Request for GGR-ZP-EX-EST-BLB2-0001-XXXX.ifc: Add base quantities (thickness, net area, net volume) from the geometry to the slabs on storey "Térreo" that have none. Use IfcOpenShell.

First a look at what the model holds.

```python
import ifcopenshell
import ifcopenshell.util.element
import ifcopenshell.util.unit

model = ifcopenshell.open("GGR-ZP-EX-EST-BLB2-0001-XXXX.ifc")
print(model.schema)
for unit_type in ("LENGTHUNIT", "AREAUNIT", "VOLUMEUNIT"):
    print(unit_type, ifcopenshell.util.unit.calculate_unit_scale(model, unit_type))
storey = next(s for s in model.by_type("IfcBuildingStorey") if s.Name == "Térreo")
slabs = [e for e in ifcopenshell.util.element.get_decomposition(storey) if e.is_a("IfcSlab")]
for e in sorted(slabs, key=lambda e: e.id()):
    print(e.id(), e.is_a(), e.Name, list(ifcopenshell.util.element.get_psets(e, qtos_only=True)), sep=" | ")
```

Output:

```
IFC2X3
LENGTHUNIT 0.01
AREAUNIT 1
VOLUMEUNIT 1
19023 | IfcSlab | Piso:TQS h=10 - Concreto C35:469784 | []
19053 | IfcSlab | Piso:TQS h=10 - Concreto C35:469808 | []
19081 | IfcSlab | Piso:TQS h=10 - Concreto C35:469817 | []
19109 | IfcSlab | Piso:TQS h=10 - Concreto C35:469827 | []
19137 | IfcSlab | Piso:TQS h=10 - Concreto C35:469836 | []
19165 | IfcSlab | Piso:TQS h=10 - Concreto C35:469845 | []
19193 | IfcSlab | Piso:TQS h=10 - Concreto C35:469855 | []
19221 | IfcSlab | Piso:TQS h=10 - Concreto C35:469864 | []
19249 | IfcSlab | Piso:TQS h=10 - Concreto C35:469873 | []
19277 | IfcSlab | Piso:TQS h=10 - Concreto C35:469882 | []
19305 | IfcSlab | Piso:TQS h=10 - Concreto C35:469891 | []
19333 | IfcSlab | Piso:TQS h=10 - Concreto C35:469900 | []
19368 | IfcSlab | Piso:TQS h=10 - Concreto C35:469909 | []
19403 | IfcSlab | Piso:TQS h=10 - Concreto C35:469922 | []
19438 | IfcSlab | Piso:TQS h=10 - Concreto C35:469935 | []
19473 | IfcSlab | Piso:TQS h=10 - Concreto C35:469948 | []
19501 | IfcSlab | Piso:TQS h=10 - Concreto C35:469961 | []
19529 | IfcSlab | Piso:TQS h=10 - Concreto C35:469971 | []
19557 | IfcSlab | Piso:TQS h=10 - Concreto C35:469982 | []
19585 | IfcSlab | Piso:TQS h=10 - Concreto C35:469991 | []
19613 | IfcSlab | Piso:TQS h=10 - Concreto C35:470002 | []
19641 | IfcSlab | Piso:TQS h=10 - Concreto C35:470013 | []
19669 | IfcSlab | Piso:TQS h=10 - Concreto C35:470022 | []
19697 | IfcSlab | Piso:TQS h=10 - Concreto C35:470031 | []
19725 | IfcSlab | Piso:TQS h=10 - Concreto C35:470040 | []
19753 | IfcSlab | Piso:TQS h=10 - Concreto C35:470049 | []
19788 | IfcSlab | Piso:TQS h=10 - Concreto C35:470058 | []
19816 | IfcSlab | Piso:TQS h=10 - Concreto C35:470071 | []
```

```python
import ifcopenshell
import ifcopenshell.api.pset
import ifcopenshell.geom
import ifcopenshell.util.element
import ifcopenshell.util.shape
import ifcopenshell.util.unit

model = ifcopenshell.open("GGR-ZP-EX-EST-BLB2-0001-XXXX.ifc")
unit_scale = ifcopenshell.util.unit.calculate_unit_scale(model)
area_scale = ifcopenshell.util.unit.calculate_unit_scale(model, "AREAUNIT")
volume_scale = ifcopenshell.util.unit.calculate_unit_scale(model, "VOLUMEUNIT")
settings = ifcopenshell.geom.settings()

storey = next(s for s in model.by_type("IfcBuildingStorey") if s.Name == "Térreo")
slabs = [e for e in ifcopenshell.util.element.get_decomposition(storey) if e.is_a("IfcSlab")]

for e in sorted(slabs, key=lambda e: e.id()):
    if ifcopenshell.util.element.get_psets(e, qtos_only=True, should_inherit=False):
        continue
    # Geometry comes back in metres, in the element's own axes.
    shape = ifcopenshell.geom.create_shape(settings, e)
    values = {
        "Width": ifcopenshell.util.shape.get_z(shape.geometry) / unit_scale,
        "NetArea": ifcopenshell.util.shape.get_footprint_area(shape.geometry) / area_scale,
        "NetVolume": ifcopenshell.util.shape.get_volume(shape.geometry) / volume_scale,
    }
    qto = ifcopenshell.api.pset.add_qto(model, product=e, name="BaseQuantities")
    ifcopenshell.api.pset.edit_qto(model, qto=qto, properties=values)
    print(e.id(), {k: round(v, 3) for k, v in values.items()})

model.write("GGR-ZP-EX-EST-BLB2-0001-XXXX_edited.ifc")
```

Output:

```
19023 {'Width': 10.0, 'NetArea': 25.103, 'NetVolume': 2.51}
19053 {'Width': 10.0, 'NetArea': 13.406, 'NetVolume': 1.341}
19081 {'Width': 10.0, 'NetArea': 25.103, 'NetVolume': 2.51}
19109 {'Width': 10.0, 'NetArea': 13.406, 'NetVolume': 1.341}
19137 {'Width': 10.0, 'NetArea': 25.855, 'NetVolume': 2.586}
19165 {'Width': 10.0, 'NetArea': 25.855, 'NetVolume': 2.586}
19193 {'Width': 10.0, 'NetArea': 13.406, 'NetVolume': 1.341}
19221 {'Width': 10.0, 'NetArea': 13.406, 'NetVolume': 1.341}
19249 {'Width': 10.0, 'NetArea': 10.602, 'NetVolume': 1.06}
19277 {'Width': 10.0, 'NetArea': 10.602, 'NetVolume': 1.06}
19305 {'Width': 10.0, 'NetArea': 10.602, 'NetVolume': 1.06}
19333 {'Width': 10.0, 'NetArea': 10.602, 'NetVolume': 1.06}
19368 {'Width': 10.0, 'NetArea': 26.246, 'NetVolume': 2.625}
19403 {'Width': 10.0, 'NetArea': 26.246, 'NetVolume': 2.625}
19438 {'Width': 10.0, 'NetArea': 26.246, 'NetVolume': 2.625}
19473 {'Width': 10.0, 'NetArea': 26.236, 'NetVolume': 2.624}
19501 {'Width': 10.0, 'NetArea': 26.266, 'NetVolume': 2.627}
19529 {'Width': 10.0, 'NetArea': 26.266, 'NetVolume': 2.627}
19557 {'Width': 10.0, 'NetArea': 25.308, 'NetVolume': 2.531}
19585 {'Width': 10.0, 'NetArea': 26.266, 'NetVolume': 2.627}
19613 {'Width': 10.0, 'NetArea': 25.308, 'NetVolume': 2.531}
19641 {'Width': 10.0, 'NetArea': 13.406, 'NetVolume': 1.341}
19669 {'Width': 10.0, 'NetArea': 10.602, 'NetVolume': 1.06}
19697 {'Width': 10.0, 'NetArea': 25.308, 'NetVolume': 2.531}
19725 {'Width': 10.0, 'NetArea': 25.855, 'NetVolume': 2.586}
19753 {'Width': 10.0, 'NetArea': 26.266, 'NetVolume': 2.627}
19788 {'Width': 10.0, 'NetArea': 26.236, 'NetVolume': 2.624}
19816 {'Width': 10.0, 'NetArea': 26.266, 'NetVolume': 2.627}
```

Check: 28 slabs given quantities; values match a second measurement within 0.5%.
